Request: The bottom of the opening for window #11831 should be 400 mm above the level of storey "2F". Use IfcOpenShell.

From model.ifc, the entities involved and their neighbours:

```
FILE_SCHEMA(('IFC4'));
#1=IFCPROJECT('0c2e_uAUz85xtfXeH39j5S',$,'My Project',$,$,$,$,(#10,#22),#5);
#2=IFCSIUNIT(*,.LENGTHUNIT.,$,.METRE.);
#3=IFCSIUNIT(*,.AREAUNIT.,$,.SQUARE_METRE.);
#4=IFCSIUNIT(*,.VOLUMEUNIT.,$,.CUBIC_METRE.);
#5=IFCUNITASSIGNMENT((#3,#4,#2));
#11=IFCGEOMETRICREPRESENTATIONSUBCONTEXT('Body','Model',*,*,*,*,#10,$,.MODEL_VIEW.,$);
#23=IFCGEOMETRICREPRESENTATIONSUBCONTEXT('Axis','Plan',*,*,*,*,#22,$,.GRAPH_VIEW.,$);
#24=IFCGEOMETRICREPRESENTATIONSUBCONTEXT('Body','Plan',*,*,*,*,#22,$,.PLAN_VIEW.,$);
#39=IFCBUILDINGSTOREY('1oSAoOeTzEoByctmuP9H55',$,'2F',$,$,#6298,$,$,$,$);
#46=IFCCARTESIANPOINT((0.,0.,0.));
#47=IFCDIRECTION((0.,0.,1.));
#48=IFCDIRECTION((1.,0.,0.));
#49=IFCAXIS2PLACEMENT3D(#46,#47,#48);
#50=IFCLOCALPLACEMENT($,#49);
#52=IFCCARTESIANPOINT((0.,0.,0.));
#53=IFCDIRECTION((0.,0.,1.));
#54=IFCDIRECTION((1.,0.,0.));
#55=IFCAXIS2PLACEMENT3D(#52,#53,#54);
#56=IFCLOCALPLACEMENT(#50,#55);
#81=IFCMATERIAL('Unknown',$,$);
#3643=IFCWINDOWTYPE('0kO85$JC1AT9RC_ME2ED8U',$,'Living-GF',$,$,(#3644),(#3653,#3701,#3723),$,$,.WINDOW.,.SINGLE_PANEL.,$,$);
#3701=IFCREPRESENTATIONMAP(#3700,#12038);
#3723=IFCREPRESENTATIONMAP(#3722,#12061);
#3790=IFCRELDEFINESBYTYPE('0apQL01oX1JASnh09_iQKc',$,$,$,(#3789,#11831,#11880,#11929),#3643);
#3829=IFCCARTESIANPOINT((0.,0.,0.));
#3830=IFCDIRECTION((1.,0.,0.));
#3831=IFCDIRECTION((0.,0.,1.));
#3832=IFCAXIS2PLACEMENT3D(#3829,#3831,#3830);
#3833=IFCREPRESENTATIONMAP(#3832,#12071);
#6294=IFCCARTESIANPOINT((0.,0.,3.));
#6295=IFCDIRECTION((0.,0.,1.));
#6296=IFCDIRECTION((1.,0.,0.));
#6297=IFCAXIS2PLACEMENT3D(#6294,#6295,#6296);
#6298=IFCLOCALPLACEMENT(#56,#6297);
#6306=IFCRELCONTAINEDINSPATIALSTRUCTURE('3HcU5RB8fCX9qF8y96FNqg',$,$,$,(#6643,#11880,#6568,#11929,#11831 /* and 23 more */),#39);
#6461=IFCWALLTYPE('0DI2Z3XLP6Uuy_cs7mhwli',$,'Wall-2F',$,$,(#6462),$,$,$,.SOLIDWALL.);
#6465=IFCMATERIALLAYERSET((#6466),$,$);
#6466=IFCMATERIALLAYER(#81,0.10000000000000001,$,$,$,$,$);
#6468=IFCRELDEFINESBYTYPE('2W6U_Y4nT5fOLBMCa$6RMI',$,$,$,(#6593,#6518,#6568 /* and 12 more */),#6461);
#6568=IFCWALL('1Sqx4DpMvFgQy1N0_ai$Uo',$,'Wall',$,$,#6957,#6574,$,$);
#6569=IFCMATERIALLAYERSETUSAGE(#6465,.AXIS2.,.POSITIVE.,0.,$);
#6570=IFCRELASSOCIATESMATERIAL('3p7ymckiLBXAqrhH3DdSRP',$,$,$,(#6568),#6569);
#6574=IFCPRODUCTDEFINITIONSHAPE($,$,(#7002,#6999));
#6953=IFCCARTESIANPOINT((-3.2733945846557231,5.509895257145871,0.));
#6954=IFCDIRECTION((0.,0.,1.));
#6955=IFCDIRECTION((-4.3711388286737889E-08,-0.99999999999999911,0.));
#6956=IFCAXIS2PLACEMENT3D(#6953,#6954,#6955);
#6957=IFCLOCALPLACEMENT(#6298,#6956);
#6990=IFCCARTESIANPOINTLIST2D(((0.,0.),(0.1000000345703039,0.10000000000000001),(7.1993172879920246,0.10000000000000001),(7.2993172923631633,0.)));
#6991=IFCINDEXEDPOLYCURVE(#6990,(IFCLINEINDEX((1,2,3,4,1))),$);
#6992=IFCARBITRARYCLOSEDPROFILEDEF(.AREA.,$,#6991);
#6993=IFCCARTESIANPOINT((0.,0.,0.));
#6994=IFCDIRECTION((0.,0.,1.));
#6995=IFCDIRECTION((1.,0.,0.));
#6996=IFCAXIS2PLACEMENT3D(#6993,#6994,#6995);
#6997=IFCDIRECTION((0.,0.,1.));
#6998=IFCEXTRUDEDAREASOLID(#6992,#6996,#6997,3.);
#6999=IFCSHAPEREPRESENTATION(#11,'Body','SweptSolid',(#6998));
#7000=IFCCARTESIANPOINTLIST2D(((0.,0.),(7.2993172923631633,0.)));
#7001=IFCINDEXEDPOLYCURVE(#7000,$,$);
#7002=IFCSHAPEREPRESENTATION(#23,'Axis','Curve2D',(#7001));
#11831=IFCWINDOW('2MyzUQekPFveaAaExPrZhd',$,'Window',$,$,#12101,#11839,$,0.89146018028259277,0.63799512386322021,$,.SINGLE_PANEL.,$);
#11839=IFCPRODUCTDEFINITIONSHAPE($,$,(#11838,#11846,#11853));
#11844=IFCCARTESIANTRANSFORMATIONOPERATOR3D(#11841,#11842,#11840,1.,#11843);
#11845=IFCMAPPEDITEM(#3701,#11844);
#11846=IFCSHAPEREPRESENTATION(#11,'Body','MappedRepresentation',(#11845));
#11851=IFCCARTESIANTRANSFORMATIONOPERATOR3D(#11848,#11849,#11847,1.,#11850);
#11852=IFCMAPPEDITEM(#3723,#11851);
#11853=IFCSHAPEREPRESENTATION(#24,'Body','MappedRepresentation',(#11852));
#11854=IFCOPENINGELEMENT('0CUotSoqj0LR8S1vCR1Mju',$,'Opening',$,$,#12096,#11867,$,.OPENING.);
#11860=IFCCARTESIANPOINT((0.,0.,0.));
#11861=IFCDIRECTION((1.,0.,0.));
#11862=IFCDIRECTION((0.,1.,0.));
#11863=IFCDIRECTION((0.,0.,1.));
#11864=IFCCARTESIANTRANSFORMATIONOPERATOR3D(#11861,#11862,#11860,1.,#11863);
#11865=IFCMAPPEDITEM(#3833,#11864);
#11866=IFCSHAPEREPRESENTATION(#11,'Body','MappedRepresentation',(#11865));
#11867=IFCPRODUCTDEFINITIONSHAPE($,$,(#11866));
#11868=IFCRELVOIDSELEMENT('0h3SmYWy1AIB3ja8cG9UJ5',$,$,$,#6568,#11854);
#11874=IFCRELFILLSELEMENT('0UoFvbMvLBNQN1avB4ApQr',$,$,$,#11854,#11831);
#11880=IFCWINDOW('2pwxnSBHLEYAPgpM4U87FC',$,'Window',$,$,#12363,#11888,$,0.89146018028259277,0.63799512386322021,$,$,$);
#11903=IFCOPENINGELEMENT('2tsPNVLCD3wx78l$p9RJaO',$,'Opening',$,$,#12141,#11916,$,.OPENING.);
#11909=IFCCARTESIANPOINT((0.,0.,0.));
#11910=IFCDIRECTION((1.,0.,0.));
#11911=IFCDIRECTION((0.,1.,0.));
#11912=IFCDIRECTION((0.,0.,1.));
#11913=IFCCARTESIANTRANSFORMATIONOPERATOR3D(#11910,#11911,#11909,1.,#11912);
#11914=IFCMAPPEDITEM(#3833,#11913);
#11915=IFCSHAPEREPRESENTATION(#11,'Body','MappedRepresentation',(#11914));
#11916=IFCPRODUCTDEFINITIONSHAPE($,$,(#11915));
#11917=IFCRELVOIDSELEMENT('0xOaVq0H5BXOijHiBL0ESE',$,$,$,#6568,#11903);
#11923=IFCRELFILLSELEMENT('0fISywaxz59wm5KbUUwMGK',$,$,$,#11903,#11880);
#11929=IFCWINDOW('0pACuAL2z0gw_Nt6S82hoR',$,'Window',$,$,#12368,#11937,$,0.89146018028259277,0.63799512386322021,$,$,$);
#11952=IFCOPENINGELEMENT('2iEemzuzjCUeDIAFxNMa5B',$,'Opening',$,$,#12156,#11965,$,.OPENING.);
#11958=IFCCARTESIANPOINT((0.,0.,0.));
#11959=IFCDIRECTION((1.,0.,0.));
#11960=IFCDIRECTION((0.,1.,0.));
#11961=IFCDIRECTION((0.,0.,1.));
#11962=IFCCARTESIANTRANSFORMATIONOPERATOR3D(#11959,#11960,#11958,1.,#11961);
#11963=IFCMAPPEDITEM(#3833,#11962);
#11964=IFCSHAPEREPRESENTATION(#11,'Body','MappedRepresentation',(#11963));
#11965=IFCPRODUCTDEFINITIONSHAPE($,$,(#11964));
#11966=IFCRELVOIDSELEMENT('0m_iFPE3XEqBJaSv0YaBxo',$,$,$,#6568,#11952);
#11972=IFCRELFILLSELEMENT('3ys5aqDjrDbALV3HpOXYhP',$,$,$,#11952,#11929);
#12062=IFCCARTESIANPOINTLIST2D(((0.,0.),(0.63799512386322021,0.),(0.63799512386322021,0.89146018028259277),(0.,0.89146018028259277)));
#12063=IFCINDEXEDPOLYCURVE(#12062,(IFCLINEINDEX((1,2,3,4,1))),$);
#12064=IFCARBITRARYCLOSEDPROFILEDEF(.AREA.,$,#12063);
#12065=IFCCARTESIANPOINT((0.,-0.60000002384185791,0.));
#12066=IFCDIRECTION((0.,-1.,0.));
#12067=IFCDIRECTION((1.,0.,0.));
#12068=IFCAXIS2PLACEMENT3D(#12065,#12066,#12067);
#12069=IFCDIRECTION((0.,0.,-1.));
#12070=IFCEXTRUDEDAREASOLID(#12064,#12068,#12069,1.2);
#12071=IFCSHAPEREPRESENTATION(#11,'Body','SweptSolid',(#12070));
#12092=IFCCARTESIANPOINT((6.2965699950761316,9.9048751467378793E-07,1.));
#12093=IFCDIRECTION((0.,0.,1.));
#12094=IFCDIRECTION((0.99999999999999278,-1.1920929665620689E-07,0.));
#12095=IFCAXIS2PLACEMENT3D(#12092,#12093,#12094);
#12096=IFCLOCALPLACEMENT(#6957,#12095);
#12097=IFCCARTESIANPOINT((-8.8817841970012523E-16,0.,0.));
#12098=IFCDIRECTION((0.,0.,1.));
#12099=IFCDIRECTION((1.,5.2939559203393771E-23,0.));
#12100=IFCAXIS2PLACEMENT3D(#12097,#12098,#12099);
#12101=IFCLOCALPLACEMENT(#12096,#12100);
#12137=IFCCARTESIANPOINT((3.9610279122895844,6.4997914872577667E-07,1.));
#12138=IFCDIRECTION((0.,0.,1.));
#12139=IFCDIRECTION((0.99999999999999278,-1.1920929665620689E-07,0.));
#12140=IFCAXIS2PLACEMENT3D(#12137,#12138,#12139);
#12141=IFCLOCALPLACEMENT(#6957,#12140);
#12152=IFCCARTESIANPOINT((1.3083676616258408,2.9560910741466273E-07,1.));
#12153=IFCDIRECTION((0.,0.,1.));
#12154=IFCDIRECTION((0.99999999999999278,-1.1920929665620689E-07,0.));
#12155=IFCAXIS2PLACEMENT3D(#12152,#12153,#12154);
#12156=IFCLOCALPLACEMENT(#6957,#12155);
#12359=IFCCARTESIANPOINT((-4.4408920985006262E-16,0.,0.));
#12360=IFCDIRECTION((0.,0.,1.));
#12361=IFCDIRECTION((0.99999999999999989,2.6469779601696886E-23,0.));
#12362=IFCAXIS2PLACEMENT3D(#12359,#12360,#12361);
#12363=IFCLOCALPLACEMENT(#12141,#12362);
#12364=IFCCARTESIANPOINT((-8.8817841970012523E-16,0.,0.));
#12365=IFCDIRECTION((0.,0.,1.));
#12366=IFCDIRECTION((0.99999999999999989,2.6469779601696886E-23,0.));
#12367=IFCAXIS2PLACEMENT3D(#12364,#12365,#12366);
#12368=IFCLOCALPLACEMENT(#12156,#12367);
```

```python
import numpy as np
import ifcopenshell
import ifcopenshell.api.geometry
import ifcopenshell.geom
import ifcopenshell.util.element
import ifcopenshell.util.placement
import ifcopenshell.util.shape
import ifcopenshell.util.unit

model = ifcopenshell.open("model.ifc")
unit_scale = ifcopenshell.util.unit.calculate_unit_scale(model)

window = model.by_guid("2MyzUQekPFveaAaExPrZhd")
opening = window.FillsVoids[0].RelatingOpeningElement
storey = ifcopenshell.util.element.get_container(window, ifc_class="IfcBuildingStorey")
level = ifcopenshell.util.placement.get_local_placement(storey.ObjectPlacement)[2, 3]

# The opening's origin need not be at the sill, so measure its lowest point.
shape = ifcopenshell.geom.create_shape(ifcopenshell.geom.settings(), opening)
bottom = ifcopenshell.util.shape.get_shape_bottom_elevation(shape, shape.geometry) / unit_scale
dz = level + 0.4 / unit_scale - bottom

shift = np.array([0.0, 0.0, dz])
# The window is placed relative to its opening, so it follows when the opening moves.
matrix = ifcopenshell.util.placement.get_local_placement(opening.ObjectPlacement)
matrix[:3, 3] += shift
ifcopenshell.api.geometry.edit_object_placement(
    model, product=opening, matrix=matrix, is_si=False, should_transform_children=True
)

print(f"moved by {dz * unit_scale:+.3f} m")

model.write("model_rev.ifc")
```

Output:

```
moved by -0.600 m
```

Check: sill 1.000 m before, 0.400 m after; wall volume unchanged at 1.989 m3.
